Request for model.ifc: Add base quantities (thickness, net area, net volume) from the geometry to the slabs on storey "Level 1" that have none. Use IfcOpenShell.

First a look at what the model holds.

```python
import ifcopenshell
import ifcopenshell.util.element
import ifcopenshell.util.unit

model = ifcopenshell.open("model.ifc")
print(model.schema)
for unit_type in ("LENGTHUNIT", "AREAUNIT", "VOLUMEUNIT"):
    print(unit_type, ifcopenshell.util.unit.calculate_unit_scale(model, unit_type))
storey = next(s for s in model.by_type("IfcBuildingStorey") if s.Name == "Level 1")
slabs = [e for e in ifcopenshell.util.element.get_decomposition(storey) if e.is_a("IfcSlab")]
for e in sorted(slabs, key=lambda e: e.id()):
    print(e.id(), e.is_a(), e.Name, list(ifcopenshell.util.element.get_psets(e, qtos_only=True)), sep=" | ")
```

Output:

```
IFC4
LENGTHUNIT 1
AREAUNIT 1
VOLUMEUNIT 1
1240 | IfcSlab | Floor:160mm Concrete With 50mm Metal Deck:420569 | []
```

```python
import ifcopenshell
import ifcopenshell.api.pset
import ifcopenshell.geom
import ifcopenshell.util.element
import ifcopenshell.util.shape
import ifcopenshell.util.unit

model = ifcopenshell.open("model.ifc")
unit_scale = ifcopenshell.util.unit.calculate_unit_scale(model)
area_scale = ifcopenshell.util.unit.calculate_unit_scale(model, "AREAUNIT")
volume_scale = ifcopenshell.util.unit.calculate_unit_scale(model, "VOLUMEUNIT")
settings = ifcopenshell.geom.settings()

storey = next(s for s in model.by_type("IfcBuildingStorey") if s.Name == "Level 1")
slabs = [e for e in ifcopenshell.util.element.get_decomposition(storey) if e.is_a("IfcSlab")]

for e in sorted(slabs, key=lambda e: e.id()):
    if ifcopenshell.util.element.get_psets(e, qtos_only=True, should_inherit=False):
        continue
    # Geometry comes back in metres, in the element's own axes.
    shape = ifcopenshell.geom.create_shape(settings, e)
    values = {
        "Width": ifcopenshell.util.shape.get_z(shape.geometry) / unit_scale,
        "NetArea": ifcopenshell.util.shape.get_footprint_area(shape.geometry) / area_scale,
        "NetVolume": ifcopenshell.util.shape.get_volume(shape.geometry) / volume_scale,
    }
    qto = ifcopenshell.api.pset.add_qto(model, product=e, name="Qto_SlabBaseQuantities")
    ifcopenshell.api.pset.edit_qto(model, qto=qto, properties=values)
    print(e.id(), {k: round(v, 3) for k, v in values.items()})

model.write("model_edited.ifc")
```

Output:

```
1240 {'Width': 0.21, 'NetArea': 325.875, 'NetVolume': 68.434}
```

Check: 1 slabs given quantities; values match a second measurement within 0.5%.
